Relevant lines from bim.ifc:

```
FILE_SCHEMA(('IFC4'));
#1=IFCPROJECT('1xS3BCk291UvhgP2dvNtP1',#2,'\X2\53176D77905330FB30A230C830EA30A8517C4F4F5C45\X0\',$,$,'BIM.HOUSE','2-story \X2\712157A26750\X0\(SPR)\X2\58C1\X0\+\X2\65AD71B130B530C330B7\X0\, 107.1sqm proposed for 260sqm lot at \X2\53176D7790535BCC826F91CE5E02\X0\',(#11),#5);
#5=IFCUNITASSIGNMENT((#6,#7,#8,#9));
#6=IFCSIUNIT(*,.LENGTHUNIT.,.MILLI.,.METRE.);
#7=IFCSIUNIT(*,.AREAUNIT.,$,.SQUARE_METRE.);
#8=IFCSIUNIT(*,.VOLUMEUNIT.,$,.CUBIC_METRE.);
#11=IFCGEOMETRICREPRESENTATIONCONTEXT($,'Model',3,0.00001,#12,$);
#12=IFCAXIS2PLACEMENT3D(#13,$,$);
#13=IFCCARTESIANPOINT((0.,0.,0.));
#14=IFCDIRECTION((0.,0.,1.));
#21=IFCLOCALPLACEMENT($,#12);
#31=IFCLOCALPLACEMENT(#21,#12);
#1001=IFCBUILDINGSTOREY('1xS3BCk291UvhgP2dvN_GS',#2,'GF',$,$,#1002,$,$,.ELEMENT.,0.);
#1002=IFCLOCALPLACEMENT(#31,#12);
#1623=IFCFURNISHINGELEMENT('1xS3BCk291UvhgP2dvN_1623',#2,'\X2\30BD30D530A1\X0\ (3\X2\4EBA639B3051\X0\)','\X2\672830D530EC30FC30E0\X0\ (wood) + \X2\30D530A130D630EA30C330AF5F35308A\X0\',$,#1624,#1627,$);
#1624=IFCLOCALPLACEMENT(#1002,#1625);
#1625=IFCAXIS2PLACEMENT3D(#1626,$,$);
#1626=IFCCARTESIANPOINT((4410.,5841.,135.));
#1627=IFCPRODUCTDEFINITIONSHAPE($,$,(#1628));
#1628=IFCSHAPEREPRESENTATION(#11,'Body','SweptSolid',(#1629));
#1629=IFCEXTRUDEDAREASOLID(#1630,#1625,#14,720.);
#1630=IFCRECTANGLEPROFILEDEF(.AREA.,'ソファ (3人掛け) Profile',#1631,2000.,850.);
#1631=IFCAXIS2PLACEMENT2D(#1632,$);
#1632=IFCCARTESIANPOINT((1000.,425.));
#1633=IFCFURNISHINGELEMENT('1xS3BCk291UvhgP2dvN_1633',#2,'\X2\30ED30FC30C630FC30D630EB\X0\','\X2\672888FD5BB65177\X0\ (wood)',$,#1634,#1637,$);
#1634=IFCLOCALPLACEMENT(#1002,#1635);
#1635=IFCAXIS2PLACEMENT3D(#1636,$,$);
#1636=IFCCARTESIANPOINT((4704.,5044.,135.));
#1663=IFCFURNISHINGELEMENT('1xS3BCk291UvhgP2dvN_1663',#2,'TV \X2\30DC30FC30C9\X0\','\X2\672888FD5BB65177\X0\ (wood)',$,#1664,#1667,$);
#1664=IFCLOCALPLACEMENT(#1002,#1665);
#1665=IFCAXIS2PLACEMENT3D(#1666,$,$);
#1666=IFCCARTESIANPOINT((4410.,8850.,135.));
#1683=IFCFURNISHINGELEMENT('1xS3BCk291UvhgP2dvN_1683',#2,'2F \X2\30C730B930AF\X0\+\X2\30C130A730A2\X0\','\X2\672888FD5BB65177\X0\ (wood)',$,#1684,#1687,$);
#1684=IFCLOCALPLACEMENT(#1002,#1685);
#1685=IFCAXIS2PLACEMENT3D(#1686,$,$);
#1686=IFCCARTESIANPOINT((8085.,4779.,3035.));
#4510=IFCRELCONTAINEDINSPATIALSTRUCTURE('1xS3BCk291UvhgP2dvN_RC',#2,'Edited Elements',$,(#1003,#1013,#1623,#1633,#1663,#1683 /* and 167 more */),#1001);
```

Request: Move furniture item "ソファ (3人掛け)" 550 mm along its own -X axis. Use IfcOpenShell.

```python
import ifcopenshell
import ifcopenshell.api.geometry
import ifcopenshell.util.placement

model = ifcopenshell.open("bim.ifc")

item = model.by_guid("1xS3BCk291UvhgP2dvN_1623")
matrix = ifcopenshell.util.placement.get_local_placement(item.ObjectPlacement)
matrix[:3, 3] -= matrix[:3, 0] * 550.0
ifcopenshell.api.geometry.edit_object_placement(model, product=item, matrix=matrix, is_si=False)

print(ifcopenshell.util.placement.get_local_placement(item.ObjectPlacement).round(3) + 0.0)

model.write("bim-out.ifc")
```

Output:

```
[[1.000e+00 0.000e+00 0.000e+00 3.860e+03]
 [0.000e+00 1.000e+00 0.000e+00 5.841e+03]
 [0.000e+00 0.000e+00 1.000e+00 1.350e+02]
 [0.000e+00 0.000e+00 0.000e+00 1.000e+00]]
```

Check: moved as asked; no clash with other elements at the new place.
